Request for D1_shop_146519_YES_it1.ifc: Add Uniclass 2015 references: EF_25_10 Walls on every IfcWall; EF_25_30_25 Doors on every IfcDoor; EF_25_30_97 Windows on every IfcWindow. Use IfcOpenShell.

First a look at what the model holds.

```python
import ifcopenshell

model = ifcopenshell.open("D1_shop_146519_YES_it1.ifc")
print(model.schema)
print("classifications:", [c.Name for c in model.by_type("IfcClassification")])
for ifc_class in ("IfcDoor", "IfcRoof", "IfcStair", "IfcWall", "IfcWindow"):
    print(ifc_class, len(model.by_type(ifc_class)))
```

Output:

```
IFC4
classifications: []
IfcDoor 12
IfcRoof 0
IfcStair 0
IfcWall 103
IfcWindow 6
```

```python
import ifcopenshell
import ifcopenshell.api.classification

model = ifcopenshell.open("D1_shop_146519_YES_it1.ifc")

system = ifcopenshell.api.classification.add_classification(model, classification="Uniclass 2015")

codes = {
    "IfcWall": ("EF_25_10", "Walls"),
    "IfcDoor": ("EF_25_30_25", "Doors"),
    "IfcWindow": ("EF_25_30_97", "Windows"),
}
for ifc_class, (code, name) in codes.items():
    products = model.by_type(ifc_class)
    ifcopenshell.api.classification.add_reference(
        model, products=products, classification=system, identification=code, name=name
    )
    print(code, len(products))

model.write("D1_shop_146519_YES_it1_edited.ifc")
```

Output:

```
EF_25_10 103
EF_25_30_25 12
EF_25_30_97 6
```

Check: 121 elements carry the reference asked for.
